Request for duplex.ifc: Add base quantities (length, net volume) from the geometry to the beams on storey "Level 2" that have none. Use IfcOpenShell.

First a look at what the model holds.

```python
import ifcopenshell
import ifcopenshell.util.element
import ifcopenshell.util.unit

model = ifcopenshell.open("duplex.ifc")
print(model.schema)
for unit_type in ("LENGTHUNIT", "AREAUNIT", "VOLUMEUNIT"):
    print(unit_type, ifcopenshell.util.unit.calculate_unit_scale(model, unit_type))
storey = next(s for s in model.by_type("IfcBuildingStorey") if s.Name == "Level 2")
beams = [e for e in ifcopenshell.util.element.get_decomposition(storey) if e.is_a("IfcBeam")]
for e in sorted(beams, key=lambda e: e.id()):
    print(e.id(), e.is_a(), e.Name, list(ifcopenshell.util.element.get_psets(e, qtos_only=True)), sep=" | ")
```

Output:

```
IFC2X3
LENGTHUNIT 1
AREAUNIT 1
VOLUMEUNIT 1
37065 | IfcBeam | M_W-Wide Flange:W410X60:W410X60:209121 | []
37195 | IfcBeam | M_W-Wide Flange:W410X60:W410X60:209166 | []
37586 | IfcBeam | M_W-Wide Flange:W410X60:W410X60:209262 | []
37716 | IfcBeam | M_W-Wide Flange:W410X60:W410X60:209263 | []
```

```python
import ifcopenshell
import ifcopenshell.api.pset
import ifcopenshell.geom
import ifcopenshell.util.element
import ifcopenshell.util.shape
import ifcopenshell.util.unit

model = ifcopenshell.open("duplex.ifc")
unit_scale = ifcopenshell.util.unit.calculate_unit_scale(model)
volume_scale = ifcopenshell.util.unit.calculate_unit_scale(model, "VOLUMEUNIT")
settings = ifcopenshell.geom.settings()

storey = next(s for s in model.by_type("IfcBuildingStorey") if s.Name == "Level 2")
beams = [e for e in ifcopenshell.util.element.get_decomposition(storey) if e.is_a("IfcBeam")]

for e in sorted(beams, key=lambda e: e.id()):
    if ifcopenshell.util.element.get_psets(e, qtos_only=True, should_inherit=False):
        continue
    # Geometry comes back in metres, in the element's own axes.
    shape = ifcopenshell.geom.create_shape(settings, e)
    values = {
        "Length": ifcopenshell.util.shape.get_max_xyz(shape.geometry) / unit_scale,
        "NetVolume": ifcopenshell.util.shape.get_volume(shape.geometry) / volume_scale,
    }
    qto = ifcopenshell.api.pset.add_qto(model, product=e, name="BaseQuantities")
    ifcopenshell.api.pset.edit_qto(model, qto=qto, properties=values)
    print(e.id(), {k: round(v, 3) for k, v in values.items()})

model.write("duplex_updated.ifc")
```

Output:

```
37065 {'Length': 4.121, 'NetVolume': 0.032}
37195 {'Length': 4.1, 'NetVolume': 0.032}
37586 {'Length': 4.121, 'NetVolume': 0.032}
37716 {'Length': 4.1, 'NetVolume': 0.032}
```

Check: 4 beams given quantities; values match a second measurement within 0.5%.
